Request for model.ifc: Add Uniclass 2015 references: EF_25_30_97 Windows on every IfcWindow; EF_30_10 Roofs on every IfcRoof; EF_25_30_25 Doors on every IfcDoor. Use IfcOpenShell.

First a look at what the model holds.

```python
import ifcopenshell

model = ifcopenshell.open("model.ifc")
print(model.schema)
print("classifications:", [c.Name for c in model.by_type("IfcClassification")])
for ifc_class in ("IfcDoor", "IfcRoof", "IfcStair", "IfcWall", "IfcWindow"):
    print(ifc_class, len(model.by_type(ifc_class)))
```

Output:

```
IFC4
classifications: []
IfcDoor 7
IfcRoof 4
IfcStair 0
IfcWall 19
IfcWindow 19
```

```python
import ifcopenshell
import ifcopenshell.api.classification

model = ifcopenshell.open("model.ifc")

system = ifcopenshell.api.classification.add_classification(model, classification="Uniclass 2015")

codes = {
    "IfcWindow": ("EF_25_30_97", "Windows"),
    "IfcRoof": ("EF_30_10", "Roofs"),
    "IfcDoor": ("EF_25_30_25", "Doors"),
}
for ifc_class, (code, name) in codes.items():
    products = model.by_type(ifc_class)
    ifcopenshell.api.classification.add_reference(
        model, products=products, classification=system, identification=code, name=name
    )
    print(code, len(products))

model.write("model_updated.ifc")
```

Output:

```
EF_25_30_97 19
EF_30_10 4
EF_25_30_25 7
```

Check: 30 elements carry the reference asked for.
